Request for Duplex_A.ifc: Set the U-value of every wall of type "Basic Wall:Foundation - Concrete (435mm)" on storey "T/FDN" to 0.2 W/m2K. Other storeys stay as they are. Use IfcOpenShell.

First a look at what the model holds.

```python
import ifcopenshell
import ifcopenshell.util.element

model = ifcopenshell.open("Duplex_A.ifc")
print(model.schema)
storey = next(s for s in model.by_type("IfcBuildingStorey") if s.Name == "T/FDN")
walls = [e for e in ifcopenshell.util.element.get_decomposition(storey) if e.is_a("IfcWall")]
seen = {}
for e in walls:
    element_type = ifcopenshell.util.element.get_type(e)
    key = (element_type.Name if element_type != e and element_type else None, ifcopenshell.util.element.get_pset(e, "Pset_WallCommon", "ThermalTransmittance"))
    seen[key] = seen.get(key, 0) + 1
for (name, value), count in sorted(seen.items(), key=str):
    print(count, "x", name, "|", value)
```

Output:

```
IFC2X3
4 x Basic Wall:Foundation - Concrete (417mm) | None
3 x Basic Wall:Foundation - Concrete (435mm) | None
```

```python
import ifcopenshell
import ifcopenshell.api.pset
import ifcopenshell.util.element

model = ifcopenshell.open("Duplex_A.ifc")

storey = next(s for s in model.by_type("IfcBuildingStorey") if s.Name == "T/FDN")
walls = [e for e in ifcopenshell.util.element.get_decomposition(storey) if e.is_a("IfcWall")]

count = 0
for e in walls:
    element_type = ifcopenshell.util.element.get_type(e)
    if element_type in (None, e) or element_type.Name != "Basic Wall:Foundation - Concrete (435mm)":
        continue
    # add_pset returns the element's existing set when there is one.
    pset = ifcopenshell.api.pset.add_pset(model, product=e, name="Pset_WallCommon")
    ifcopenshell.api.pset.edit_pset(model, pset=pset, properties={"ThermalTransmittance": 0.2})
    count += 1

print(count, "walls updated")

model.write("Duplex_A-out.ifc")
```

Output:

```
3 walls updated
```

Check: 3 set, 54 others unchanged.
